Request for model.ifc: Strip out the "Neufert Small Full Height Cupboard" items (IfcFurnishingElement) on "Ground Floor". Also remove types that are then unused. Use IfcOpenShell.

First a look at what the model holds.

```python
import ifcopenshell
import ifcopenshell.util.element

model = ifcopenshell.open("model.ifc")
print(model.schema)
storey = next(s for s in model.by_type("IfcBuildingStorey") if s.Name == "Ground Floor")
furniture = [e for e in ifcopenshell.util.element.get_decomposition(storey) if e.is_a("IfcFurnishingElement")]
seen = {}
for e in furniture:
    element_type = ifcopenshell.util.element.get_type(e)
    name = element_type.Name if element_type not in (None, e) else None
    seen[name] = seen.get(name, 0) + 1
for name, count in sorted(seen.items(), key=str):
    print(count, "x", name)
```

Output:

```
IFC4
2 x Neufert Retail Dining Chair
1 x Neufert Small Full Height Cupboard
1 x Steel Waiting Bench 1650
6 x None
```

```python
import ifcopenshell
import ifcopenshell.api.root
import ifcopenshell.util.element

model = ifcopenshell.open("model.ifc")

storey = next(s for s in model.by_type("IfcBuildingStorey") if s.Name == "Ground Floor")
furniture = [e for e in ifcopenshell.util.element.get_decomposition(storey) if e.is_a("IfcFurnishingElement")]
targets = [e for e in furniture if (t := ifcopenshell.util.element.get_type(e)) not in (None, e) and t.Name == "Neufert Small Full Height Cupboard"]
types = {ifcopenshell.util.element.get_type(e) for e in targets} - {None, *targets}

for e in targets:
    ifcopenshell.api.root.remove_product(model, product=e)
print(len(targets), "removed")

unused = [t for t in types if not ifcopenshell.util.element.get_types(t)]
for t in unused:
    ifcopenshell.api.root.remove_product(model, product=t)
print(len(unused), "unused types removed")

model.write("model-out.ifc")
```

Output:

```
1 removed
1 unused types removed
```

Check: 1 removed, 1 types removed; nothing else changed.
